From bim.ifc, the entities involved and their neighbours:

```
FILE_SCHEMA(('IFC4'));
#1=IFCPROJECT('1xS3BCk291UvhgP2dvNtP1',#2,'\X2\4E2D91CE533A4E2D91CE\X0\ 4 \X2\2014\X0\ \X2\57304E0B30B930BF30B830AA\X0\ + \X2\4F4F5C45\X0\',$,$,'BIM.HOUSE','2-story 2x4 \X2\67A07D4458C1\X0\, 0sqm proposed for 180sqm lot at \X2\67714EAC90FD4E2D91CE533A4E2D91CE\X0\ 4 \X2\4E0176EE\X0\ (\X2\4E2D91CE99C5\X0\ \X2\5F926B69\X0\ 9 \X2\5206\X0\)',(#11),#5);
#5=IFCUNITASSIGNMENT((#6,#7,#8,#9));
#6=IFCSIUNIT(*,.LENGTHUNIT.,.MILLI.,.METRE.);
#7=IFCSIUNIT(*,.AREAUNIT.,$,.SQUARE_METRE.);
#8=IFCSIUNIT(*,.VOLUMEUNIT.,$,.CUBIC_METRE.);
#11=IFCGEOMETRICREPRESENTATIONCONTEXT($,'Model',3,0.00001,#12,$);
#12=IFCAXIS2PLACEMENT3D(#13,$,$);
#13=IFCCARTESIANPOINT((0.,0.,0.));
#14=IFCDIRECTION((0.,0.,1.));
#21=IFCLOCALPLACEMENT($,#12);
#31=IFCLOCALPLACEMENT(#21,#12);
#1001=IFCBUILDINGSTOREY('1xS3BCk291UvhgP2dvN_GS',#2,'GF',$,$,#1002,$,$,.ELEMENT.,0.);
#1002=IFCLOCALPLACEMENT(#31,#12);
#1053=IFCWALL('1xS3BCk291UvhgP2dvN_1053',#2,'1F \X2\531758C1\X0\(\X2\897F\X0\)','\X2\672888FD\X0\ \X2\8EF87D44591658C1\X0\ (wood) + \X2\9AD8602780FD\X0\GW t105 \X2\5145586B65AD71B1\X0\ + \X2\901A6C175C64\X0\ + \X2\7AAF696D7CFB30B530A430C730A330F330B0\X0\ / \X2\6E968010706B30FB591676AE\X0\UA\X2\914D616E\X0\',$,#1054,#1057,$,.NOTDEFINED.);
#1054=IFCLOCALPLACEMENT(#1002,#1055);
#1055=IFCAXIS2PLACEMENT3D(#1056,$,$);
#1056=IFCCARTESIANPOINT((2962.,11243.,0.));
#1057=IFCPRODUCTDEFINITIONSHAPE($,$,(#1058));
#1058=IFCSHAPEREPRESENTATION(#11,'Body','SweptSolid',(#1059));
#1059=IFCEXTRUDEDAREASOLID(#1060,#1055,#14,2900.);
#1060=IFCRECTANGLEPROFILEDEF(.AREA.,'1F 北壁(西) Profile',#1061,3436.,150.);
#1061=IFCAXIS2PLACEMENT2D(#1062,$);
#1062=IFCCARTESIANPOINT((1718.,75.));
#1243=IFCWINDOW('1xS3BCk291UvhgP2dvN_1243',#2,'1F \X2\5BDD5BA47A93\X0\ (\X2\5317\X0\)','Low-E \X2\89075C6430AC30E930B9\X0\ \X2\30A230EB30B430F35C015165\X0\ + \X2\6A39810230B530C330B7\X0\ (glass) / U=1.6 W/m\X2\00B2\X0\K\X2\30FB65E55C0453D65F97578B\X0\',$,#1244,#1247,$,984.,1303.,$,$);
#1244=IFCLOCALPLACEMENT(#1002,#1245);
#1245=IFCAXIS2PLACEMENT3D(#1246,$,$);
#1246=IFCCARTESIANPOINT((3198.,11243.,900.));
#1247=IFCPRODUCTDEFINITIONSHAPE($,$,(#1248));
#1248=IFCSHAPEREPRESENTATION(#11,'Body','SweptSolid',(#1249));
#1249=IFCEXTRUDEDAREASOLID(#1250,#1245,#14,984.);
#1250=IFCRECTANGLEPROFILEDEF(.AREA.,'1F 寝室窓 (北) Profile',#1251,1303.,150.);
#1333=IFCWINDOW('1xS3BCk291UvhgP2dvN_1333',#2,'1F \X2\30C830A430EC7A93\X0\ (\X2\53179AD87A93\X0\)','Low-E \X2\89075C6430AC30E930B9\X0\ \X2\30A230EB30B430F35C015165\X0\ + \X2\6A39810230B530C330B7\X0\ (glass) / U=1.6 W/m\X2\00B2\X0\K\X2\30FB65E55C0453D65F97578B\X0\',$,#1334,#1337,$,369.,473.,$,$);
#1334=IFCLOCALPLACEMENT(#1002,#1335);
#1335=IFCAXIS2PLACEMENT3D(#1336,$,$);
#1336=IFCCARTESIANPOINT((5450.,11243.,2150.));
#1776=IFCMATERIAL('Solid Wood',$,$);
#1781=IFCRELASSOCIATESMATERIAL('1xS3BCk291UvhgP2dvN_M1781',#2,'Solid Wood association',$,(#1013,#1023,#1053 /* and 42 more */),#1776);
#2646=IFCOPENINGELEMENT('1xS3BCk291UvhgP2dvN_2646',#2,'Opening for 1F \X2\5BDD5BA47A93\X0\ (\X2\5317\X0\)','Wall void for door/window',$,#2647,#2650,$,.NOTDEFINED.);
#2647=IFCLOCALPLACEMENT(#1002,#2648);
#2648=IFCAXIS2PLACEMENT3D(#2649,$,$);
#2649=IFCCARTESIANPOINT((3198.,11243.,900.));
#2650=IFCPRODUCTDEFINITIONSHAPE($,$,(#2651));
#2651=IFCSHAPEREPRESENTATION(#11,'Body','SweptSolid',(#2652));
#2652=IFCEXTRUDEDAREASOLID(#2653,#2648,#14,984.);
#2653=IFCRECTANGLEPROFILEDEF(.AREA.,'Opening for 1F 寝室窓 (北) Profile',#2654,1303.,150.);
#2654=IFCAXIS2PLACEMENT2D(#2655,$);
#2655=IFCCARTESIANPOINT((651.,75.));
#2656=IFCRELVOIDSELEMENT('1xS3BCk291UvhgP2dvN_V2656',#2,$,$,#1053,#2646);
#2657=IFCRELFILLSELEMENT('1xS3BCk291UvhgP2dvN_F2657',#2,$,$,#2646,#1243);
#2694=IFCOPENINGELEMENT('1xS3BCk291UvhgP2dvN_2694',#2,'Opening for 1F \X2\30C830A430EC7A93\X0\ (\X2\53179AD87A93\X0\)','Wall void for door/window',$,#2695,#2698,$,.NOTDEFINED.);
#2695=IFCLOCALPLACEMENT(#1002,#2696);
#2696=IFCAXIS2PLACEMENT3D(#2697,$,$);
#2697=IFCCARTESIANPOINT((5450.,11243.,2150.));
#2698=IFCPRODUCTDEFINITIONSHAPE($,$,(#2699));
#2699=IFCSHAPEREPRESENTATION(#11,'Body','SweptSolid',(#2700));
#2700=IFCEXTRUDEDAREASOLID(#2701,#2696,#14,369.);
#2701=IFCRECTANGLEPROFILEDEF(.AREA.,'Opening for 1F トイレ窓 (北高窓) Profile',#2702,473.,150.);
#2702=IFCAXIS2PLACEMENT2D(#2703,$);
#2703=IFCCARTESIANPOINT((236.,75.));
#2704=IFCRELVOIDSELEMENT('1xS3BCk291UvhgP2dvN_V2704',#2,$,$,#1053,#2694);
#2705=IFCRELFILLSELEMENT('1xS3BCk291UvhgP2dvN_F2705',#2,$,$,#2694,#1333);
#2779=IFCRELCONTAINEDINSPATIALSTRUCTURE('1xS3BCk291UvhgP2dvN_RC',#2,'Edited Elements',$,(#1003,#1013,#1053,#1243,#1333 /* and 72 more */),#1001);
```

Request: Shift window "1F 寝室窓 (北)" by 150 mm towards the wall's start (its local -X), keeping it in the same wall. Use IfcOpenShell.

```python
import ifcopenshell
import ifcopenshell.api.geometry
import ifcopenshell.util.placement

model = ifcopenshell.open("bim.ifc")

window = model.by_guid("1xS3BCk291UvhgP2dvN_1243")
opening = window.FillsVoids[0].RelatingOpeningElement
wall = opening.VoidsElements[0].RelatingBuildingElement

wall_matrix = ifcopenshell.util.placement.get_local_placement(wall.ObjectPlacement)
shift = wall_matrix[:3, 0] * -150.0
before = ifcopenshell.util.placement.get_local_placement(window.ObjectPlacement)[:3, 3].copy()

# The window is not placed relative to its opening, so move both.
for product in (opening, window):
    matrix = ifcopenshell.util.placement.get_local_placement(product.ObjectPlacement)
    matrix[:3, 3] += shift
    ifcopenshell.api.geometry.edit_object_placement(model, product=product, matrix=matrix, is_si=False)

after = ifcopenshell.util.placement.get_local_placement(window.ObjectPlacement)[:3, 3]
print("window moved by", (after - before).round(3) + 0.0)

model.write("bim_updated.ifc")
```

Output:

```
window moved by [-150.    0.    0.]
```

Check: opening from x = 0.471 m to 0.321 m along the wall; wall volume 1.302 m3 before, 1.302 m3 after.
